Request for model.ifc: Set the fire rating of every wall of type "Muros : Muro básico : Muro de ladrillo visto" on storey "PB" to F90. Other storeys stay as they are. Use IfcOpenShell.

First a look at what the model holds.

```python
import ifcopenshell
import ifcopenshell.util.element

model = ifcopenshell.open("model.ifc")
print(model.schema)
storey = next(s for s in model.by_type("IfcBuildingStorey") if s.Name == "PB")
walls = [e for e in ifcopenshell.util.element.get_decomposition(storey) if e.is_a("IfcWall")]
seen = {}
for e in walls:
    element_type = ifcopenshell.util.element.get_type(e)
    key = (element_type.Name if element_type != e and element_type else None, ifcopenshell.util.element.get_pset(e, "Pset_WallCommon", "FireRating"))
    seen[key] = seen.get(key, 0) + 1
for (name, value), count in sorted(seen.items(), key=str):
    print(count, "x", name, "|", value)
```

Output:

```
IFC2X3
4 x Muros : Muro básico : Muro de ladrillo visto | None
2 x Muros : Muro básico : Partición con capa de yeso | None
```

```python
import ifcopenshell
import ifcopenshell.api.pset
import ifcopenshell.util.element

model = ifcopenshell.open("model.ifc")

storey = next(s for s in model.by_type("IfcBuildingStorey") if s.Name == "PB")
walls = [e for e in ifcopenshell.util.element.get_decomposition(storey) if e.is_a("IfcWall")]

count = 0
for e in walls:
    element_type = ifcopenshell.util.element.get_type(e)
    if element_type in (None, e) or element_type.Name != "Muros : Muro básico : Muro de ladrillo visto":
        continue
    # add_pset returns the element's existing set when there is one.
    pset = ifcopenshell.api.pset.add_pset(model, product=e, name="Pset_WallCommon")
    ifcopenshell.api.pset.edit_pset(model, pset=pset, properties={"FireRating": "F90"})
    count += 1

print(count, "walls updated")

model.write("model-out.ifc")
```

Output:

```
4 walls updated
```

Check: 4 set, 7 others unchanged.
